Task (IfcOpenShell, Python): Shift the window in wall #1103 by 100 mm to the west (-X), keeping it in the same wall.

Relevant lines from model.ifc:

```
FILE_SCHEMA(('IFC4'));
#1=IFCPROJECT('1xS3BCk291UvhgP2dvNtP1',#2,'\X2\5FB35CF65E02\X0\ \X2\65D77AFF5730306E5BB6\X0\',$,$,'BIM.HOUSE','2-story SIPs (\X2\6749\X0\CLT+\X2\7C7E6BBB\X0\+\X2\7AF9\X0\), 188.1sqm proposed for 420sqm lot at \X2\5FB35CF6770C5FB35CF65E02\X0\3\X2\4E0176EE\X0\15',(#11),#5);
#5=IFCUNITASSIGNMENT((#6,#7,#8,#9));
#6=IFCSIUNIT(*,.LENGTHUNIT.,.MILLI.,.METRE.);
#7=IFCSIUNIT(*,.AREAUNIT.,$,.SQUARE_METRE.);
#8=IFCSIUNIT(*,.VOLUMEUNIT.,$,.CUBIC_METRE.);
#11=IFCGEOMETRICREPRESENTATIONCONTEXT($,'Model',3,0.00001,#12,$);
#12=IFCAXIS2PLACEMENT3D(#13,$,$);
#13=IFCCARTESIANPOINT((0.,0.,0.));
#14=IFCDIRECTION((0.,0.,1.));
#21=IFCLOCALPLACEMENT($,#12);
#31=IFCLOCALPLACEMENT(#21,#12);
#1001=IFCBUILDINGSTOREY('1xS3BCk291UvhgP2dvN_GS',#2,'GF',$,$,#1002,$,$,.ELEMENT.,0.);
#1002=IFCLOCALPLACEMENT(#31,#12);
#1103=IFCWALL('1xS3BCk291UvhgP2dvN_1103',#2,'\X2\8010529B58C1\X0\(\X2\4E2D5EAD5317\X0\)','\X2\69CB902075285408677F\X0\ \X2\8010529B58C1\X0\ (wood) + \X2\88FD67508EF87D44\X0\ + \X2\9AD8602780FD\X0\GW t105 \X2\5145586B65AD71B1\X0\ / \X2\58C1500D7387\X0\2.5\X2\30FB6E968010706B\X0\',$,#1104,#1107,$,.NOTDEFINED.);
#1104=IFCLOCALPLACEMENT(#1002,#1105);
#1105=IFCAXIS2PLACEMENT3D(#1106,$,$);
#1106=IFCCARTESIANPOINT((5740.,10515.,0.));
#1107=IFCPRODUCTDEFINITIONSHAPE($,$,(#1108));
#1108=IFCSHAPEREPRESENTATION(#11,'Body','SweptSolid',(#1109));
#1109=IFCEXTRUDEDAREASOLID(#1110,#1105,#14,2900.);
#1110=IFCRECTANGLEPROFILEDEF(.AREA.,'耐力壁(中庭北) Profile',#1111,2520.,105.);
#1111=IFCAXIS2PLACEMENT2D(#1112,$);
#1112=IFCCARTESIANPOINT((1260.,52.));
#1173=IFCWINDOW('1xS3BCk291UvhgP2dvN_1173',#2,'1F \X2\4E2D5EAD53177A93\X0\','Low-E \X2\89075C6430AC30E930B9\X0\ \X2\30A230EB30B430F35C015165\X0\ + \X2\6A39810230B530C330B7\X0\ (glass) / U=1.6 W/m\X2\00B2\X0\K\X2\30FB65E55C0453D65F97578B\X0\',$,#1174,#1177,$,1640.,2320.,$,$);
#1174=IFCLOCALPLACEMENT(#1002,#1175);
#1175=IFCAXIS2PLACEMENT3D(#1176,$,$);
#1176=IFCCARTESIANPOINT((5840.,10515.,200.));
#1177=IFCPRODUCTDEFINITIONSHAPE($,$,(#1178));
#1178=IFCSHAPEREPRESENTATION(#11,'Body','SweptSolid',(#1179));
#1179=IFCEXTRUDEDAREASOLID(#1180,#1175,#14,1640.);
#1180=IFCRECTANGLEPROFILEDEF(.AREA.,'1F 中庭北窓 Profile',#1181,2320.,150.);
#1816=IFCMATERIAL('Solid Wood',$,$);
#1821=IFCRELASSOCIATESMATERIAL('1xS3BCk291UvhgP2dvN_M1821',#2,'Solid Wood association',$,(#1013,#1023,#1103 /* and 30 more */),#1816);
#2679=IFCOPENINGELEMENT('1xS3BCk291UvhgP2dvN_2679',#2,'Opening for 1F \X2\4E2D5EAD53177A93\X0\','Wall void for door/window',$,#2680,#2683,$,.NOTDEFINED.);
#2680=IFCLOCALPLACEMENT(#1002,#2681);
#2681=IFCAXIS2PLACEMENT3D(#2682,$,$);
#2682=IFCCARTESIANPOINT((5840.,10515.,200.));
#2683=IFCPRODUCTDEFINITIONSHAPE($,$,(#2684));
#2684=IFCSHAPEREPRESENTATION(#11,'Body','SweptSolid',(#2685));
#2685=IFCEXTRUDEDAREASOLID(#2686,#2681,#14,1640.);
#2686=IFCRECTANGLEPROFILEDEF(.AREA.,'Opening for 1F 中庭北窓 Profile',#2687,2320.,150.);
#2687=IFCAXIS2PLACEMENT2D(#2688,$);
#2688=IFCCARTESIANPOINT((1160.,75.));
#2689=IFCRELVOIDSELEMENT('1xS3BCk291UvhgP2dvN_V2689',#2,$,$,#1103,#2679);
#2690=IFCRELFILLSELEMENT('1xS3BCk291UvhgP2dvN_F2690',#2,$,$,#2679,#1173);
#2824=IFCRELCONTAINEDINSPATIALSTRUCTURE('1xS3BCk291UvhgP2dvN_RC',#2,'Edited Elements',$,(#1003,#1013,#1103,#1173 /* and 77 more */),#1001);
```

```python
import ifcopenshell
import ifcopenshell.api.geometry
import ifcopenshell.util.placement
import ifcopenshell.util.unit

model = ifcopenshell.open("model.ifc")
unit_scale = ifcopenshell.util.unit.calculate_unit_scale(model)

window = model.by_id(1173)
opening = window.FillsVoids[0].RelatingOpeningElement
wall = opening.VoidsElements[0].RelatingBuildingElement

wall_matrix = ifcopenshell.util.placement.get_local_placement(wall.ObjectPlacement)
shift = wall_matrix[:3, 0] * -0.1 / unit_scale
before = ifcopenshell.util.placement.get_local_placement(window.ObjectPlacement)[:3, 3].copy()

# The window is not placed relative to its opening, so move both.
for product in (opening, window):
    matrix = ifcopenshell.util.placement.get_local_placement(product.ObjectPlacement)
    matrix[:3, 3] += shift
    ifcopenshell.api.geometry.edit_object_placement(model, product=product, matrix=matrix, is_si=False)

after = ifcopenshell.util.placement.get_local_placement(window.ObjectPlacement)[:3, 3]
print("window moved by", (after - before).round(3) + 0.0)

model.write("model_rev.ifc")
```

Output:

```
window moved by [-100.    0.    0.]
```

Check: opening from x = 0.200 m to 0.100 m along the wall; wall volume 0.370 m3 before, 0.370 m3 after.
